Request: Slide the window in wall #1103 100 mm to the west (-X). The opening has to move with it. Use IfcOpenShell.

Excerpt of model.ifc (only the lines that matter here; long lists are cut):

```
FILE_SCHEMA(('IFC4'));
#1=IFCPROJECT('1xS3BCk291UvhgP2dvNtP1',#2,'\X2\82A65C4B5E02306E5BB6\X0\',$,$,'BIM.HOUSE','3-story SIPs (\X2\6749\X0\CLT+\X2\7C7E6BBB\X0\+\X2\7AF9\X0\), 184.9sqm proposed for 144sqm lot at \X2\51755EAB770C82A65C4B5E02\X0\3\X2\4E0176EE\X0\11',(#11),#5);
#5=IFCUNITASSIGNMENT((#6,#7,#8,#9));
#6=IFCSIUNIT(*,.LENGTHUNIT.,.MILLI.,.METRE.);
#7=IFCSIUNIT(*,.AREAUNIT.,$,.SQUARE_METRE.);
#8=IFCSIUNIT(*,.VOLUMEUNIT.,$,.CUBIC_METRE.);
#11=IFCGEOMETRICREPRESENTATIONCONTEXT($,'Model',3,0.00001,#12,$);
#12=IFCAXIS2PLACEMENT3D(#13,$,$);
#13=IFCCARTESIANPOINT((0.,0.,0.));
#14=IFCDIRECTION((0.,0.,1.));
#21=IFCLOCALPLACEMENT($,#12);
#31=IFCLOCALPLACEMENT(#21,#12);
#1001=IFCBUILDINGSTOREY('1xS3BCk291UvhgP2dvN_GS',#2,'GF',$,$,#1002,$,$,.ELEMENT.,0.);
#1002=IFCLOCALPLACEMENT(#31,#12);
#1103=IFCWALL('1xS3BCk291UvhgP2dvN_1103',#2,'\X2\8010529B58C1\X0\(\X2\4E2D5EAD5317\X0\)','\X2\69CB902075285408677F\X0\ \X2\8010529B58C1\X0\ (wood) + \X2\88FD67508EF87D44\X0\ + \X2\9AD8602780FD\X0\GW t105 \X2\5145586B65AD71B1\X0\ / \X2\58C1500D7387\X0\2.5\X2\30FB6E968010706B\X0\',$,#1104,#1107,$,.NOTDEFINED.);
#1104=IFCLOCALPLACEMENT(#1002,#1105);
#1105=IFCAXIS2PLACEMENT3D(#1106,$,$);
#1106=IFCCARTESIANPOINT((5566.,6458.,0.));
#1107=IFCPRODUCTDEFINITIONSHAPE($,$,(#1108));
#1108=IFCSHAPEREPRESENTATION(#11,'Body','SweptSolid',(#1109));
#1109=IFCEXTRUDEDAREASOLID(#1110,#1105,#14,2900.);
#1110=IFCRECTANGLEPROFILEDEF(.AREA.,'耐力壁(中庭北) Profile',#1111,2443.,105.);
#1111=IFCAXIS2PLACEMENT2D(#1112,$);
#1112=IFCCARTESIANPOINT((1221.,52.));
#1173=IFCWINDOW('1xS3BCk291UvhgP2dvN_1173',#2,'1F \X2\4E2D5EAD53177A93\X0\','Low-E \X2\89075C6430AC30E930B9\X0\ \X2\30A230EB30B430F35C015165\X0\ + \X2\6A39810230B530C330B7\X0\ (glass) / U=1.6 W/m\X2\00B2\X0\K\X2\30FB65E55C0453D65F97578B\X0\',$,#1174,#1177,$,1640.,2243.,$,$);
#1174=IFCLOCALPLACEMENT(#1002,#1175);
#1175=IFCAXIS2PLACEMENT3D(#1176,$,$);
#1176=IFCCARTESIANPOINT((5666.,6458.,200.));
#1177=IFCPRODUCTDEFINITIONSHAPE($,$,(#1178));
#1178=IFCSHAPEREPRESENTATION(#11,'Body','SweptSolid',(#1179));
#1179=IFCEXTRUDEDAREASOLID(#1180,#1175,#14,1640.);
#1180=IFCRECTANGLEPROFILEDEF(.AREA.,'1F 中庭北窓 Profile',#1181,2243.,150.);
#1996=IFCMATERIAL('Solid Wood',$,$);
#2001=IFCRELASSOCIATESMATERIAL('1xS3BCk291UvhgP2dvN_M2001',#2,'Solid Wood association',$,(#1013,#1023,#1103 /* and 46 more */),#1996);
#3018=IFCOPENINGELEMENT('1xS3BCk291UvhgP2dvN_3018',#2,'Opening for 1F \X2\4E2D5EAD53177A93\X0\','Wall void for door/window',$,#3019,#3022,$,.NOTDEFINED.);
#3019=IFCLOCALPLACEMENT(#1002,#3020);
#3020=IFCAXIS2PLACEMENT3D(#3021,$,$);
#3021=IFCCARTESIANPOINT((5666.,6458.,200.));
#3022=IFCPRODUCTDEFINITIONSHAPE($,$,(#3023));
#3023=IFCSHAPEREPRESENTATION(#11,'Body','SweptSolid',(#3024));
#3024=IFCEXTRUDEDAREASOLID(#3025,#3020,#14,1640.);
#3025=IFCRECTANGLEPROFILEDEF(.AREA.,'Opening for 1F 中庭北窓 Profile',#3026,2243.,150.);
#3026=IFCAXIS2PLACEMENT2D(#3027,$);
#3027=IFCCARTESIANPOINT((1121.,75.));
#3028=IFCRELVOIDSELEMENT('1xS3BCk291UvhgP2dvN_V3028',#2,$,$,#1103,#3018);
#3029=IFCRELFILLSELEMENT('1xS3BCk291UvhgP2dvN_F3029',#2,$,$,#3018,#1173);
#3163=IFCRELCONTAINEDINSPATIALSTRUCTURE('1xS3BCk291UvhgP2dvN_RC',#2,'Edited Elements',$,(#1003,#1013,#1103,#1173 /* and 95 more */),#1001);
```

```python
import ifcopenshell
import ifcopenshell.api.geometry
import ifcopenshell.util.placement
import ifcopenshell.util.unit

model = ifcopenshell.open("model.ifc")
unit_scale = ifcopenshell.util.unit.calculate_unit_scale(model)

window = model.by_guid("1xS3BCk291UvhgP2dvN_1173")
opening = window.FillsVoids[0].RelatingOpeningElement
wall = opening.VoidsElements[0].RelatingBuildingElement

wall_matrix = ifcopenshell.util.placement.get_local_placement(wall.ObjectPlacement)
shift = wall_matrix[:3, 0] * -0.1 / unit_scale
before = ifcopenshell.util.placement.get_local_placement(window.ObjectPlacement)[:3, 3].copy()

# The window is not placed relative to its opening, so move both.
for product in (opening, window):
    matrix = ifcopenshell.util.placement.get_local_placement(product.ObjectPlacement)
    matrix[:3, 3] += shift
    ifcopenshell.api.geometry.edit_object_placement(model, product=product, matrix=matrix, is_si=False)

after = ifcopenshell.util.placement.get_local_placement(window.ObjectPlacement)[:3, 3]
print("window moved by", (after - before).round(3) + 0.0)

model.write("model_updated.ifc")
```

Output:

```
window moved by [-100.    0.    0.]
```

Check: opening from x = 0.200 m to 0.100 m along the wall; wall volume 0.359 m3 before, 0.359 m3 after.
